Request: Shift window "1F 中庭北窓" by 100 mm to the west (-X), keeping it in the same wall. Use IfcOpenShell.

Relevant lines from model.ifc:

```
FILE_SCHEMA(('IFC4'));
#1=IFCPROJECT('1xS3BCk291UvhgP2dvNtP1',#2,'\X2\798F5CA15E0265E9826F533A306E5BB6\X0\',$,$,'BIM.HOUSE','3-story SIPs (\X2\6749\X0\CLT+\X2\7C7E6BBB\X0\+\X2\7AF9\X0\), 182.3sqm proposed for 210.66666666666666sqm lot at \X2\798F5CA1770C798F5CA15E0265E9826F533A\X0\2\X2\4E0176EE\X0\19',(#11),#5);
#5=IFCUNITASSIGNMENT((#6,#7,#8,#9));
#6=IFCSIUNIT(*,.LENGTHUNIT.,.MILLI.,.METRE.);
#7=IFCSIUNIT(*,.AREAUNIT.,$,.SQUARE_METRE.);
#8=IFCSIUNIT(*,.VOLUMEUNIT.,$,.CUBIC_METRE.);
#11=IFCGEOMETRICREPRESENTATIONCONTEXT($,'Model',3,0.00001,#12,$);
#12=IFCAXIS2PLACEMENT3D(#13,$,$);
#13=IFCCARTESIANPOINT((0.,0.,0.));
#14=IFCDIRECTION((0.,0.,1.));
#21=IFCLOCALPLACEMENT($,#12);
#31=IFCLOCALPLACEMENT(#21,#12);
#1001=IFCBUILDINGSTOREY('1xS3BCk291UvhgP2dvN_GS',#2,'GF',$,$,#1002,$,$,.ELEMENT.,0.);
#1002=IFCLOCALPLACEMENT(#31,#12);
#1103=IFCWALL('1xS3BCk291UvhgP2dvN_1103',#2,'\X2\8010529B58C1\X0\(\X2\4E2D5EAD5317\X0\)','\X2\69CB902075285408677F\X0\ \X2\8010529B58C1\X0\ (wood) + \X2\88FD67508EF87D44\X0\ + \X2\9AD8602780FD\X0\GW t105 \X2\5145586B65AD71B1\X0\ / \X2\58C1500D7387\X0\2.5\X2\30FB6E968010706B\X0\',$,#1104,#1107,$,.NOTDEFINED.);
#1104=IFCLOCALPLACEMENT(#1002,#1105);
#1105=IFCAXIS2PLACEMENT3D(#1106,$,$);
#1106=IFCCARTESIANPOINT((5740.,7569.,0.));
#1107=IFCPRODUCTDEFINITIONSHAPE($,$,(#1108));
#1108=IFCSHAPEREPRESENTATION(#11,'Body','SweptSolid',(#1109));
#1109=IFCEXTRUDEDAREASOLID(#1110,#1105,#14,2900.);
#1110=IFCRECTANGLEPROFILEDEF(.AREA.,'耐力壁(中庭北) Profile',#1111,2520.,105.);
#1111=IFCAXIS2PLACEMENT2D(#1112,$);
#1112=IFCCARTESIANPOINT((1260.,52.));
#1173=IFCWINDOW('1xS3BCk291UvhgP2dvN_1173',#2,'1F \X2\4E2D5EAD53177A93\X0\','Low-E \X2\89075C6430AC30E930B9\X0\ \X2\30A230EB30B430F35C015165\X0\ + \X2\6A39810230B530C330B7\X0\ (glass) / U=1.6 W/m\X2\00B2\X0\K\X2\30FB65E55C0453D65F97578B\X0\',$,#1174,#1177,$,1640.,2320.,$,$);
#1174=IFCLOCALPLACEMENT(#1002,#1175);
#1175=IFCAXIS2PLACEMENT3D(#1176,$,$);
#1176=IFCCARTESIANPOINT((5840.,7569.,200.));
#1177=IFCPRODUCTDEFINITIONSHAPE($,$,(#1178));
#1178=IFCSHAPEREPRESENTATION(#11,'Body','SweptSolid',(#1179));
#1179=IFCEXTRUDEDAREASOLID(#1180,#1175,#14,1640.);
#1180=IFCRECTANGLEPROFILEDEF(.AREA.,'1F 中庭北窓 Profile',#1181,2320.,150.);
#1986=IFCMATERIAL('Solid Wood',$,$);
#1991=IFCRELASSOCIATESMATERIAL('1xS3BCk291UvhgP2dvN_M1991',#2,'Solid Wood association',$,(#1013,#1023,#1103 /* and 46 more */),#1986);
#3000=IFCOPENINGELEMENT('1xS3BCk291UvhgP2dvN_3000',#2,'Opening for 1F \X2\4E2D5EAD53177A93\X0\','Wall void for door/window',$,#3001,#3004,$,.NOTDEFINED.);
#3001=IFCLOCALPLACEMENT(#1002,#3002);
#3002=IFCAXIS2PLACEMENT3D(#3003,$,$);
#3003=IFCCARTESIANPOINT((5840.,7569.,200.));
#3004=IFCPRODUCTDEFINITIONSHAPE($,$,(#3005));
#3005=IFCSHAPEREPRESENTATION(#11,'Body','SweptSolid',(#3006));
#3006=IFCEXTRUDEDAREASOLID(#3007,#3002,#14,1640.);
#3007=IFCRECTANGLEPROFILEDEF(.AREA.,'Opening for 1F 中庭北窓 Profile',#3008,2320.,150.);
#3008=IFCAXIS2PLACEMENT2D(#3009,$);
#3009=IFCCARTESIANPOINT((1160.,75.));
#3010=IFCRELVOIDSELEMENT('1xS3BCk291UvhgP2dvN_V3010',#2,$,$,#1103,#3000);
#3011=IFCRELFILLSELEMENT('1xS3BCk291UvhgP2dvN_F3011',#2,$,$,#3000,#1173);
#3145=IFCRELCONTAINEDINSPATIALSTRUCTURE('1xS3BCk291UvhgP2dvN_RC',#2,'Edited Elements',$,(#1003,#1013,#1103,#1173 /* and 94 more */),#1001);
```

```python
import ifcopenshell
import ifcopenshell.api.geometry
import ifcopenshell.util.placement

model = ifcopenshell.open("model.ifc")

window = model.by_guid("1xS3BCk291UvhgP2dvN_1173")
opening = window.FillsVoids[0].RelatingOpeningElement
wall = opening.VoidsElements[0].RelatingBuildingElement

wall_matrix = ifcopenshell.util.placement.get_local_placement(wall.ObjectPlacement)
shift = wall_matrix[:3, 0] * -100.0
before = ifcopenshell.util.placement.get_local_placement(window.ObjectPlacement)[:3, 3].copy()

# The window is not placed relative to its opening, so move both.
for product in (opening, window):
    matrix = ifcopenshell.util.placement.get_local_placement(product.ObjectPlacement)
    matrix[:3, 3] += shift
    ifcopenshell.api.geometry.edit_object_placement(model, product=product, matrix=matrix, is_si=False)

after = ifcopenshell.util.placement.get_local_placement(window.ObjectPlacement)[:3, 3]
print("window moved by", (after - before).round(3) + 0.0)

model.write("model_updated.ifc")
```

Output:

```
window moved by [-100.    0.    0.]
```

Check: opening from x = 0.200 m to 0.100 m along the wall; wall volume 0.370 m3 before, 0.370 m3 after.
